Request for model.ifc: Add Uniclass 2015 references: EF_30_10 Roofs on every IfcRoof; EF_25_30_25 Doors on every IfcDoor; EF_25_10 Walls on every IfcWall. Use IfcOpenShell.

First a look at what the model holds.

```python
import ifcopenshell

model = ifcopenshell.open("model.ifc")
print(model.schema)
print("classifications:", [c.Name for c in model.by_type("IfcClassification")])
for ifc_class in ("IfcDoor", "IfcRoof", "IfcStair", "IfcWall", "IfcWindow"):
    print(ifc_class, len(model.by_type(ifc_class)))
```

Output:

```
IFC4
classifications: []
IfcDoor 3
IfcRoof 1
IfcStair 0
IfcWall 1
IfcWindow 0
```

```python
import ifcopenshell
import ifcopenshell.api.classification

model = ifcopenshell.open("model.ifc")

system = ifcopenshell.api.classification.add_classification(model, classification="Uniclass 2015")

codes = {
    "IfcRoof": ("EF_30_10", "Roofs"),
    "IfcDoor": ("EF_25_30_25", "Doors"),
    "IfcWall": ("EF_25_10", "Walls"),
}
for ifc_class, (code, name) in codes.items():
    products = model.by_type(ifc_class)
    ifcopenshell.api.classification.add_reference(
        model, products=products, classification=system, identification=code, name=name
    )
    print(code, len(products))

model.write("model_edited.ifc")
```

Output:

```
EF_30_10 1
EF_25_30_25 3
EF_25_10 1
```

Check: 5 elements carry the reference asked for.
